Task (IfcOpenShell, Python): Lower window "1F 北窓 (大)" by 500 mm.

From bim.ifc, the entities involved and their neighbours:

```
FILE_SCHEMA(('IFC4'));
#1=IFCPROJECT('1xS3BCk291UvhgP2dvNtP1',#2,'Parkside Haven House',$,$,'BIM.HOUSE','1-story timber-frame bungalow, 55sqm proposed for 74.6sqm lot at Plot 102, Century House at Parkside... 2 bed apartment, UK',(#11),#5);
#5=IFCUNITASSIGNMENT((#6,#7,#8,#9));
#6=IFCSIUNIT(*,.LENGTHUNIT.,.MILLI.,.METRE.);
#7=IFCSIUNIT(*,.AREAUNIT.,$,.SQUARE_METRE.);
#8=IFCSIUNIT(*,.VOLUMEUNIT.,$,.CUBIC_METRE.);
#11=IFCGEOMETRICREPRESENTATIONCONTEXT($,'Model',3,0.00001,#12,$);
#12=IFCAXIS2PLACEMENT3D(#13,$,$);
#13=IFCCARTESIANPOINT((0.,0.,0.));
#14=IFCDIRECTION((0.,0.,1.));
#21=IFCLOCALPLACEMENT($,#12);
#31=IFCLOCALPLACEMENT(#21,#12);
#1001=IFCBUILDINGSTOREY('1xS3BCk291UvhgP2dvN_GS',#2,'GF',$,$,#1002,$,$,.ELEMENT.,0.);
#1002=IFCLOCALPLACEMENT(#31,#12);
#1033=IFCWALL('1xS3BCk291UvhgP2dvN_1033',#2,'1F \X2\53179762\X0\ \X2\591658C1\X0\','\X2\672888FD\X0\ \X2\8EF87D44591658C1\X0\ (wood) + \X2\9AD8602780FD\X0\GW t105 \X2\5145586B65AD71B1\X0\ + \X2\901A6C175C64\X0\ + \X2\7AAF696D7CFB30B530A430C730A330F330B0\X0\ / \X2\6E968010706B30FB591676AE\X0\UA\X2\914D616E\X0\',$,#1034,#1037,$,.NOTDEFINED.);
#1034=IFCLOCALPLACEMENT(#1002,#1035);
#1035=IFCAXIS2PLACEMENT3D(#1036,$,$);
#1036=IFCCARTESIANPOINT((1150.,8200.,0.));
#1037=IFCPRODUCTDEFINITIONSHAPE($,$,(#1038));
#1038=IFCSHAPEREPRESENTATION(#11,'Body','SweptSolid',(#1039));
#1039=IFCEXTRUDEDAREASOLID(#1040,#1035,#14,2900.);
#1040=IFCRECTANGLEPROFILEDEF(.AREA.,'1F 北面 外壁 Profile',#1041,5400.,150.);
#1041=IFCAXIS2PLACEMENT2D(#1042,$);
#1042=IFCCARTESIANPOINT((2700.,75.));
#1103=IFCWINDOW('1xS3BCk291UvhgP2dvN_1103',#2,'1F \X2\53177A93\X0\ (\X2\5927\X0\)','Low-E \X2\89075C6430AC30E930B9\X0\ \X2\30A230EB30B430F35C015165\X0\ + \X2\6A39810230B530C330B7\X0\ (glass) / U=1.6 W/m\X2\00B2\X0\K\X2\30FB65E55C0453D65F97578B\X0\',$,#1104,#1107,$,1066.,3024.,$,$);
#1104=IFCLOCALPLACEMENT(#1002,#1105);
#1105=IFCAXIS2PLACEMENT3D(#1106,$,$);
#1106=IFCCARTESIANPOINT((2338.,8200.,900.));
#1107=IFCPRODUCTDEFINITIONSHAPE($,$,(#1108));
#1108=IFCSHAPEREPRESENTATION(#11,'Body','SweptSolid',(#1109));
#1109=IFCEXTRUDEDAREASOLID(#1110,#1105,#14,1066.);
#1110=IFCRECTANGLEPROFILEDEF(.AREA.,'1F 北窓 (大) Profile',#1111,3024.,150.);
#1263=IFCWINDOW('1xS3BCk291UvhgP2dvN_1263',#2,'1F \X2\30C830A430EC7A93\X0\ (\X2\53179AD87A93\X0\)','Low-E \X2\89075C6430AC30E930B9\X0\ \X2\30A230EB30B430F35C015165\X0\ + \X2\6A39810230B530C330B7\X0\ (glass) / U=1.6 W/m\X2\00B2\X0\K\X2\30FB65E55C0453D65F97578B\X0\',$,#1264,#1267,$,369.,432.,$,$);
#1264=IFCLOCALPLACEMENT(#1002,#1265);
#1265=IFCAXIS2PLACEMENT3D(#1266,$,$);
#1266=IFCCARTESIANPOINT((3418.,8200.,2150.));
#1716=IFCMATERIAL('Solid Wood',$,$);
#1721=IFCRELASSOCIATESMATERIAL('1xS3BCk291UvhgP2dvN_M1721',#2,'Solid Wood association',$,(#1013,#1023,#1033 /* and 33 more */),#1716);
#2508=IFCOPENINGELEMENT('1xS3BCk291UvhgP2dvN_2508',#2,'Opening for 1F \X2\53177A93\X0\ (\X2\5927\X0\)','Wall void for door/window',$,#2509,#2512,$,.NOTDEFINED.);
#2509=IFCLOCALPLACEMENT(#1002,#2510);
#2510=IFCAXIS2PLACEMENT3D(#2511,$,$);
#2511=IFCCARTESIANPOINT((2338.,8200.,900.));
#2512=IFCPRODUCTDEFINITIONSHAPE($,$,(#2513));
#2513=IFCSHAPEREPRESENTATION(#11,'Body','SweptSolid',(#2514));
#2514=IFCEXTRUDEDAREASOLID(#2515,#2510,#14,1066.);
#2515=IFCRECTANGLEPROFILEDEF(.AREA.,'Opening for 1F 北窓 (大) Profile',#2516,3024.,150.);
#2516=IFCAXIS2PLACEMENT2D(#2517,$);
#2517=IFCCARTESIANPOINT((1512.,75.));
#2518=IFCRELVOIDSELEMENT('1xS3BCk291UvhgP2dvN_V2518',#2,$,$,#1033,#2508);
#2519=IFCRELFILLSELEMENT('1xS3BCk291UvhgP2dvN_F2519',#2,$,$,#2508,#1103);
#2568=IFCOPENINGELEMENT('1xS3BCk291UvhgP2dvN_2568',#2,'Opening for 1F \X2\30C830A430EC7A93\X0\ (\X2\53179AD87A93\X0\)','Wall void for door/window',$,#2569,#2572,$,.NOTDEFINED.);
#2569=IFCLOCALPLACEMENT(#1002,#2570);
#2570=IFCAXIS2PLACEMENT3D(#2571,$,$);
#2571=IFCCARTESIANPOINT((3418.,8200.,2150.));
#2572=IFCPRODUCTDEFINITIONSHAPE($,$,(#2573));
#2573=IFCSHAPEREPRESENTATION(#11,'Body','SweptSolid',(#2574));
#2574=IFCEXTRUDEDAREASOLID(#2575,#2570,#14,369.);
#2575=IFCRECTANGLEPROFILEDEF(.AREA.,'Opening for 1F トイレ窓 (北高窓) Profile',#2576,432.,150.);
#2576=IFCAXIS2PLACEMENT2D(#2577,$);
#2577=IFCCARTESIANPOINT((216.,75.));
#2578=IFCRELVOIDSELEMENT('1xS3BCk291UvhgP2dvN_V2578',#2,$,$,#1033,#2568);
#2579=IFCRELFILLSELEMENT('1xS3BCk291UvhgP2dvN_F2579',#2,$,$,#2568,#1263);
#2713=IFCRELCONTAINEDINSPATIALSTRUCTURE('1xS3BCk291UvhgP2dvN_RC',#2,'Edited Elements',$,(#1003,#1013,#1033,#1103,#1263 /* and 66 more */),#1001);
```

```python
import numpy as np
import ifcopenshell
import ifcopenshell.api.geometry
import ifcopenshell.util.placement
import ifcopenshell.util.unit

model = ifcopenshell.open("bim.ifc")
unit_scale = ifcopenshell.util.unit.calculate_unit_scale(model)

window = model.by_guid("1xS3BCk291UvhgP2dvN_1103")
opening = window.FillsVoids[0].RelatingOpeningElement
dz = -500.0

shift = np.array([0.0, 0.0, dz])
# The window is not placed relative to its opening, so move both.
for product in (opening, window):
    matrix = ifcopenshell.util.placement.get_local_placement(product.ObjectPlacement)
    matrix[:3, 3] += shift
    ifcopenshell.api.geometry.edit_object_placement(model, product=product, matrix=matrix, is_si=False)

print(f"moved by {dz * unit_scale:+.3f} m")

model.write("bim_edited.ifc")
```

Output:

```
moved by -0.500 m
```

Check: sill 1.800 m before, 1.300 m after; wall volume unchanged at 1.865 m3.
